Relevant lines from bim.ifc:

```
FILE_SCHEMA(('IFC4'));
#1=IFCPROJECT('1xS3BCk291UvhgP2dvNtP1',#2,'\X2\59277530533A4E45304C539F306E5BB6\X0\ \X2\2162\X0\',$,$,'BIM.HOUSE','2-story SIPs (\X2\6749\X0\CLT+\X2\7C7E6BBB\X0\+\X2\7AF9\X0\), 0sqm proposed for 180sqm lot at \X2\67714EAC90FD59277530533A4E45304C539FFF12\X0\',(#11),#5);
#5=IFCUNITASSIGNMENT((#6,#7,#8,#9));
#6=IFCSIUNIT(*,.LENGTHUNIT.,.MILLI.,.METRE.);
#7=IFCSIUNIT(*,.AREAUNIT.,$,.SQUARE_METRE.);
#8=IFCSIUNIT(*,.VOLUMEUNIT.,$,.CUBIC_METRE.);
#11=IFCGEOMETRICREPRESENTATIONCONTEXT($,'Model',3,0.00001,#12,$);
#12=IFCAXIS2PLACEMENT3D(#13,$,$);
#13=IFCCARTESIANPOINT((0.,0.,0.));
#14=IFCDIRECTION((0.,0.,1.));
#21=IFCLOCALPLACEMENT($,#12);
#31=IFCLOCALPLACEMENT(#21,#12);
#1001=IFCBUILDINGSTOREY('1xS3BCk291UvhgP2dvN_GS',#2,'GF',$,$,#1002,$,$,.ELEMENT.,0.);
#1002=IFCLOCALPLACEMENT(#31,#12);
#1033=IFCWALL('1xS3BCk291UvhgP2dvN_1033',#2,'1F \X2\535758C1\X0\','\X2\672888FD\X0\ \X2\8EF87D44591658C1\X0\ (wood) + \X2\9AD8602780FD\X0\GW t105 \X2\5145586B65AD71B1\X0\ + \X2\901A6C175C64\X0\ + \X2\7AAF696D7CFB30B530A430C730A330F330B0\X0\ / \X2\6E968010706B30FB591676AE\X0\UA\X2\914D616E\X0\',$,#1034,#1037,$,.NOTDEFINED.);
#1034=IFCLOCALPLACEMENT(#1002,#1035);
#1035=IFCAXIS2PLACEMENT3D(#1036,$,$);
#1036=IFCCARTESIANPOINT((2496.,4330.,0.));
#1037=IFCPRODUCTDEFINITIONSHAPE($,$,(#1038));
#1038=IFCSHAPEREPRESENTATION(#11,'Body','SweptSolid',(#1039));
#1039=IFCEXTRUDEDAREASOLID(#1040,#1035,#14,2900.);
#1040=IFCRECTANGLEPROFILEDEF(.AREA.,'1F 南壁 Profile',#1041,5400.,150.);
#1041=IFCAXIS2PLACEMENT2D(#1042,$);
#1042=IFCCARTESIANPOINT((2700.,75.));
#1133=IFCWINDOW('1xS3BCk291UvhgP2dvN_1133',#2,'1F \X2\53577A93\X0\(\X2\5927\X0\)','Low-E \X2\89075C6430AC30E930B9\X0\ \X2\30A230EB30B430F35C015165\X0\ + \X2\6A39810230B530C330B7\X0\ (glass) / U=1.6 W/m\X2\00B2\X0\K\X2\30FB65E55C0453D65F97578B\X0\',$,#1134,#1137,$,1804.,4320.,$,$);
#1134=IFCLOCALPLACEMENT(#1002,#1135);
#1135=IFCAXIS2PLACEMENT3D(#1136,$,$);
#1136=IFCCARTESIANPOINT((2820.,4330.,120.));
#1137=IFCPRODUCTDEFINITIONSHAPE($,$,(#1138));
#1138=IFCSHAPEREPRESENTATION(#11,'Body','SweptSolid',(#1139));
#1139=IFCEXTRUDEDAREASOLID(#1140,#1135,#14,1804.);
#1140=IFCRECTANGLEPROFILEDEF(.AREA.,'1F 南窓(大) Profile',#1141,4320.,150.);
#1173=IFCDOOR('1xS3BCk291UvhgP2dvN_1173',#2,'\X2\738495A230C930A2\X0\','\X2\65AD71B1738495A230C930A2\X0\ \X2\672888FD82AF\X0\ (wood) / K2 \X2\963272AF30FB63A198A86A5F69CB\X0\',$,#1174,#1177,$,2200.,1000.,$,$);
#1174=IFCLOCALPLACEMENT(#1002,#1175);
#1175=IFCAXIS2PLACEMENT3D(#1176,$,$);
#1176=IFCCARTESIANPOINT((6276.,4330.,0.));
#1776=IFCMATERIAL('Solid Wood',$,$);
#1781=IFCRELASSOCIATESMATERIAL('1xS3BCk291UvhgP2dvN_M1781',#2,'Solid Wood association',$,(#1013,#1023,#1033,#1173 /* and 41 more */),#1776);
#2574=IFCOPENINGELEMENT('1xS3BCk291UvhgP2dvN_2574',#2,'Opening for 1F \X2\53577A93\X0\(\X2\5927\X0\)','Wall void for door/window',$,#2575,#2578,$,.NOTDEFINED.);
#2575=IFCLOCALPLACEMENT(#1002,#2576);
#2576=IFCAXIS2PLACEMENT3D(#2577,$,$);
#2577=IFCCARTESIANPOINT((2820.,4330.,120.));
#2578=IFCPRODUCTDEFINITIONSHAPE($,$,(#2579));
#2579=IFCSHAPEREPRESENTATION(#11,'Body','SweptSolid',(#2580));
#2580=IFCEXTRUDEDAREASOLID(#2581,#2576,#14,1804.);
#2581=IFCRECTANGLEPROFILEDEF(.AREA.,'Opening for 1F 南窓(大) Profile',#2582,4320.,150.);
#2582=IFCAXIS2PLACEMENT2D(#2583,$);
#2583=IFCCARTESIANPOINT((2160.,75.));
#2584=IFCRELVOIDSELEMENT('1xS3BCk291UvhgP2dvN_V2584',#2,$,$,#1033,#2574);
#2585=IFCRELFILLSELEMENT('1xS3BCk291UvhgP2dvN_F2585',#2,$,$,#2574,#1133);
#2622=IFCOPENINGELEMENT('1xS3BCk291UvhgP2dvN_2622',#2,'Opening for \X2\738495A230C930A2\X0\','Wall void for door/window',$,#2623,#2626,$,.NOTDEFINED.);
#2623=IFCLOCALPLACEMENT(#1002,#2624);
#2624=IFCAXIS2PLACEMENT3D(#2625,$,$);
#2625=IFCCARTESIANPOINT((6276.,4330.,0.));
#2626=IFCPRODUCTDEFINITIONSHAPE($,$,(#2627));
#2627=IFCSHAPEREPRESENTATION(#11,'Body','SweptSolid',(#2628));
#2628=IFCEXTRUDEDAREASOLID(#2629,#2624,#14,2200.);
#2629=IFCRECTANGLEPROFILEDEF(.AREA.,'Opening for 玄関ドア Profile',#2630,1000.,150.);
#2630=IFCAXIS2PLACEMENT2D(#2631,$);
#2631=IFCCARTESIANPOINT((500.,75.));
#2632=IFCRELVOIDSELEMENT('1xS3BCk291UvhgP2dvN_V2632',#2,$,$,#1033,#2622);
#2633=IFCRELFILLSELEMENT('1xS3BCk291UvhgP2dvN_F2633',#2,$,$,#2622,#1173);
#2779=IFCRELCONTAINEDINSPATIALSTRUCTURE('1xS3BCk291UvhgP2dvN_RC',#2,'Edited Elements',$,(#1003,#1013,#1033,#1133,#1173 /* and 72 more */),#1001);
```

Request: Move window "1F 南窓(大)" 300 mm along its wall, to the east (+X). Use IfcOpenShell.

```python
import ifcopenshell
import ifcopenshell.api.geometry
import ifcopenshell.util.placement
import ifcopenshell.util.unit

model = ifcopenshell.open("bim.ifc")
unit_scale = ifcopenshell.util.unit.calculate_unit_scale(model)

window = model.by_guid("1xS3BCk291UvhgP2dvN_1133")
opening = window.FillsVoids[0].RelatingOpeningElement
wall = opening.VoidsElements[0].RelatingBuildingElement

wall_matrix = ifcopenshell.util.placement.get_local_placement(wall.ObjectPlacement)
shift = wall_matrix[:3, 0] * 0.3 / unit_scale
before = ifcopenshell.util.placement.get_local_placement(window.ObjectPlacement)[:3, 3].copy()

# The window is not placed relative to its opening, so move both.
for product in (opening, window):
    matrix = ifcopenshell.util.placement.get_local_placement(product.ObjectPlacement)
    matrix[:3, 3] += shift
    ifcopenshell.api.geometry.edit_object_placement(model, product=product, matrix=matrix, is_si=False)

after = ifcopenshell.util.placement.get_local_placement(window.ObjectPlacement)[:3, 3]
print("window moved by", (after - before).round(3) + 0.0)

model.write("bim-out.ifc")
```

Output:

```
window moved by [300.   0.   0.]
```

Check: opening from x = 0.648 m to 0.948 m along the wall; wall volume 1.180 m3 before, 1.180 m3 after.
